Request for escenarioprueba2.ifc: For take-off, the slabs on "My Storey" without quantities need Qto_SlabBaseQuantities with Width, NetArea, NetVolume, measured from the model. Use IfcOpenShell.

First a look at what the model holds.

```python
import ifcopenshell
import ifcopenshell.util.element
import ifcopenshell.util.unit

model = ifcopenshell.open("escenarioprueba2.ifc")
print(model.schema)
for unit_type in ("LENGTHUNIT", "AREAUNIT", "VOLUMEUNIT"):
    print(unit_type, ifcopenshell.util.unit.calculate_unit_scale(model, unit_type))
storey = next(s for s in model.by_type("IfcBuildingStorey") if s.Name == "My Storey")
slabs = [e for e in ifcopenshell.util.element.get_decomposition(storey) if e.is_a("IfcSlab")]
for e in sorted(slabs, key=lambda e: e.id()):
    print(e.id(), e.is_a(), e.Name, list(ifcopenshell.util.element.get_psets(e, qtos_only=True)), sep=" | ")
```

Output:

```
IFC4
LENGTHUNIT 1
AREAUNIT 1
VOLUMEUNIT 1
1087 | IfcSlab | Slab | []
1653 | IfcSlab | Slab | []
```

```python
import ifcopenshell
import ifcopenshell.api.pset
import ifcopenshell.geom
import ifcopenshell.util.element
import ifcopenshell.util.shape
import ifcopenshell.util.unit

model = ifcopenshell.open("escenarioprueba2.ifc")
unit_scale = ifcopenshell.util.unit.calculate_unit_scale(model)
area_scale = ifcopenshell.util.unit.calculate_unit_scale(model, "AREAUNIT")
volume_scale = ifcopenshell.util.unit.calculate_unit_scale(model, "VOLUMEUNIT")
settings = ifcopenshell.geom.settings()

storey = next(s for s in model.by_type("IfcBuildingStorey") if s.Name == "My Storey")
slabs = [e for e in ifcopenshell.util.element.get_decomposition(storey) if e.is_a("IfcSlab")]

for e in sorted(slabs, key=lambda e: e.id()):
    if ifcopenshell.util.element.get_psets(e, qtos_only=True, should_inherit=False):
        continue
    # Geometry comes back in metres, in the element's own axes.
    shape = ifcopenshell.geom.create_shape(settings, e)
    values = {
        "Width": ifcopenshell.util.shape.get_z(shape.geometry) / unit_scale,
        "NetArea": ifcopenshell.util.shape.get_footprint_area(shape.geometry) / area_scale,
        "NetVolume": ifcopenshell.util.shape.get_volume(shape.geometry) / volume_scale,
    }
    qto = ifcopenshell.api.pset.add_qto(model, product=e, name="Qto_SlabBaseQuantities")
    ifcopenshell.api.pset.edit_qto(model, qto=qto, properties=values)
    print(e.id(), {k: round(v, 3) for k, v in values.items()})

model.write("escenarioprueba2-out.ifc")
```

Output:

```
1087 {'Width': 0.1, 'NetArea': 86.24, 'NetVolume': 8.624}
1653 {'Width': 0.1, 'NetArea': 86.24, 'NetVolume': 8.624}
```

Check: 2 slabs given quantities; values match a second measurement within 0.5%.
